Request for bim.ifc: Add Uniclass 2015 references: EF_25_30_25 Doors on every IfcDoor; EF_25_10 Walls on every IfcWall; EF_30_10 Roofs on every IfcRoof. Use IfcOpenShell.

First a look at what the model holds.

```python
import ifcopenshell

model = ifcopenshell.open("bim.ifc")
print(model.schema)
print("classifications:", [c.Name for c in model.by_type("IfcClassification")])
for ifc_class in ("IfcDoor", "IfcRoof", "IfcStair", "IfcWall", "IfcWindow"):
    print(ifc_class, len(model.by_type(ifc_class)))
```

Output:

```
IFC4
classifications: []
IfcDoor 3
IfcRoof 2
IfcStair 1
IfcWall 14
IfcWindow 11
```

```python
import ifcopenshell
import ifcopenshell.api.classification

model = ifcopenshell.open("bim.ifc")

system = ifcopenshell.api.classification.add_classification(model, classification="Uniclass 2015")

codes = {
    "IfcDoor": ("EF_25_30_25", "Doors"),
    "IfcWall": ("EF_25_10", "Walls"),
    "IfcRoof": ("EF_30_10", "Roofs"),
}
for ifc_class, (code, name) in codes.items():
    products = model.by_type(ifc_class)
    ifcopenshell.api.classification.add_reference(
        model, products=products, classification=system, identification=code, name=name
    )
    print(code, len(products))

model.write("bim-out.ifc")
```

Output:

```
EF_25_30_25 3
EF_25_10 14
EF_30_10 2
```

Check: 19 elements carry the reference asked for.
